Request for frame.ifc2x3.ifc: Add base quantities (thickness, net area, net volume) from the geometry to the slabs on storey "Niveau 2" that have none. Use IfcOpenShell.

First a look at what the model holds.

```python
import ifcopenshell
import ifcopenshell.util.element
import ifcopenshell.util.unit

model = ifcopenshell.open("frame.ifc2x3.ifc")
print(model.schema)
for unit_type in ("LENGTHUNIT", "AREAUNIT", "VOLUMEUNIT"):
    print(unit_type, ifcopenshell.util.unit.calculate_unit_scale(model, unit_type))
storey = next(s for s in model.by_type("IfcBuildingStorey") if s.Name == "Niveau 2")
slabs = [e for e in ifcopenshell.util.element.get_decomposition(storey) if e.is_a("IfcSlab")]
for e in sorted(slabs, key=lambda e: e.id()):
    print(e.id(), e.is_a(), e.Name, list(ifcopenshell.util.element.get_psets(e, qtos_only=True)), sep=" | ")
```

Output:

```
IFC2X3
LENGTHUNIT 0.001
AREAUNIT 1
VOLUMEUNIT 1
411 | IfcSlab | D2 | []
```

```python
import ifcopenshell
import ifcopenshell.api.pset
import ifcopenshell.geom
import ifcopenshell.util.element
import ifcopenshell.util.shape
import ifcopenshell.util.unit

model = ifcopenshell.open("frame.ifc2x3.ifc")
unit_scale = ifcopenshell.util.unit.calculate_unit_scale(model)
area_scale = ifcopenshell.util.unit.calculate_unit_scale(model, "AREAUNIT")
volume_scale = ifcopenshell.util.unit.calculate_unit_scale(model, "VOLUMEUNIT")
settings = ifcopenshell.geom.settings()

storey = next(s for s in model.by_type("IfcBuildingStorey") if s.Name == "Niveau 2")
slabs = [e for e in ifcopenshell.util.element.get_decomposition(storey) if e.is_a("IfcSlab")]

for e in sorted(slabs, key=lambda e: e.id()):
    if ifcopenshell.util.element.get_psets(e, qtos_only=True, should_inherit=False):
        continue
    # Geometry comes back in metres, in the element's own axes.
    shape = ifcopenshell.geom.create_shape(settings, e)
    values = {
        "Width": ifcopenshell.util.shape.get_z(shape.geometry) / unit_scale,
        "NetArea": ifcopenshell.util.shape.get_footprint_area(shape.geometry) / area_scale,
        "NetVolume": ifcopenshell.util.shape.get_volume(shape.geometry) / volume_scale,
    }
    qto = ifcopenshell.api.pset.add_qto(model, product=e, name="BaseQuantities")
    ifcopenshell.api.pset.edit_qto(model, qto=qto, properties=values)
    print(e.id(), {k: round(v, 3) for k, v in values.items()})

model.write("frame.ifc2x3_updated.ifc")
```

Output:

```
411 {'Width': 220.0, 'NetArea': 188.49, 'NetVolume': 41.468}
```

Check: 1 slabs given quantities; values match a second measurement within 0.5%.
